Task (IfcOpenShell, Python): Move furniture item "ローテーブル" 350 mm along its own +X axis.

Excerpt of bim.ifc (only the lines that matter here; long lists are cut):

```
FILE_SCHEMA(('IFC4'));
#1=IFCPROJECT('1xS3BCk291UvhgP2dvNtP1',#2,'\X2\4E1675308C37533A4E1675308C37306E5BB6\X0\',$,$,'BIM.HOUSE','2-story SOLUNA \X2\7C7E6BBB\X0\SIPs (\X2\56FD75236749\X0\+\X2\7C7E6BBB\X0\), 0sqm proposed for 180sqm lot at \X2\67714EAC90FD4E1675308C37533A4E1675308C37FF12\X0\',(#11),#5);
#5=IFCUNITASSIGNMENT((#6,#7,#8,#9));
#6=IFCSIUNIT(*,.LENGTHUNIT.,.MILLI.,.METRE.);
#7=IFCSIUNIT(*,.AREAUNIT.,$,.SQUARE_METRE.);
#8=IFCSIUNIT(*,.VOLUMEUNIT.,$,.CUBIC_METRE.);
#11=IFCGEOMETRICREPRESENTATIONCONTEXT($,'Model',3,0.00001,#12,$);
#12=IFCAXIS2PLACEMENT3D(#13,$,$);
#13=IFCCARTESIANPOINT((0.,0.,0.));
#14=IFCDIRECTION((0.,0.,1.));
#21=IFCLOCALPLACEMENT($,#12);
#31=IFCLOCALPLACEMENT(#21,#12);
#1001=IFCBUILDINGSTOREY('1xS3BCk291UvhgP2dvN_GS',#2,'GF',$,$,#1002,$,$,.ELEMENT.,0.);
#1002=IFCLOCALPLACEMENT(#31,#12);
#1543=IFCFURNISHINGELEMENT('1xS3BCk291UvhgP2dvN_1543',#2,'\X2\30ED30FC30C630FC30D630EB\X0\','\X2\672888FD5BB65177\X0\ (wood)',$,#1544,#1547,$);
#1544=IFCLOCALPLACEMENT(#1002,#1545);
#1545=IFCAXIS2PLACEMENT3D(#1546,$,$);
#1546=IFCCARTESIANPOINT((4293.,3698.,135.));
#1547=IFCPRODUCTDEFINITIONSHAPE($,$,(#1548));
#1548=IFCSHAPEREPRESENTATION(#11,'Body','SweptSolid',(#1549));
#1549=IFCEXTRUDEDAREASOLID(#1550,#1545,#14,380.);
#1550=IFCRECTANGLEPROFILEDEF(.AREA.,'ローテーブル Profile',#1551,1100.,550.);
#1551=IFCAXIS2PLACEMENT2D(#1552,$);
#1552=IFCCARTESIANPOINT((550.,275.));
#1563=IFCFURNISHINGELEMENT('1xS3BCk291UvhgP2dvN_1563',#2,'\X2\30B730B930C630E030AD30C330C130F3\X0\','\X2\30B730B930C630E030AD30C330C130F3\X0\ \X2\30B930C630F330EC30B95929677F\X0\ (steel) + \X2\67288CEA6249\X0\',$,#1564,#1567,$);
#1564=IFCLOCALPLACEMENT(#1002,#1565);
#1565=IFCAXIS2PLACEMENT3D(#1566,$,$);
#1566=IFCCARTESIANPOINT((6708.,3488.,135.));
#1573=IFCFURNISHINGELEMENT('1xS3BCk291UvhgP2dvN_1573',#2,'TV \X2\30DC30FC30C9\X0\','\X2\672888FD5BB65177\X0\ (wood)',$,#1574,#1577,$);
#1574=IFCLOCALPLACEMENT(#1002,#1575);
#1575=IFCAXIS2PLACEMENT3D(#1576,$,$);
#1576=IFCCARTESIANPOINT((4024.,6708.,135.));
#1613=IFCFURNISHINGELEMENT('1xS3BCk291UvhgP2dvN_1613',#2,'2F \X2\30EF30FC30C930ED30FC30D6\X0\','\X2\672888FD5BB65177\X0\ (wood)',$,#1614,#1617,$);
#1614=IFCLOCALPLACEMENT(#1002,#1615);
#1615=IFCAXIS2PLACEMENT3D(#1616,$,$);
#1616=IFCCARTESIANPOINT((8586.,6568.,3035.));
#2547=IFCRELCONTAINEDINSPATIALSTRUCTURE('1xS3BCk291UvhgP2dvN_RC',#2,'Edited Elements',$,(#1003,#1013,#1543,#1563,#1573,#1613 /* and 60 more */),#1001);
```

```python
import ifcopenshell
import ifcopenshell.api.geometry
import ifcopenshell.util.placement

model = ifcopenshell.open("bim.ifc")

item = model.by_guid("1xS3BCk291UvhgP2dvN_1543")
matrix = ifcopenshell.util.placement.get_local_placement(item.ObjectPlacement)
matrix[:3, 3] += matrix[:3, 0] * 350.0
ifcopenshell.api.geometry.edit_object_placement(model, product=item, matrix=matrix, is_si=False)

print(ifcopenshell.util.placement.get_local_placement(item.ObjectPlacement).round(3) + 0.0)

model.write("bim-out.ifc")
```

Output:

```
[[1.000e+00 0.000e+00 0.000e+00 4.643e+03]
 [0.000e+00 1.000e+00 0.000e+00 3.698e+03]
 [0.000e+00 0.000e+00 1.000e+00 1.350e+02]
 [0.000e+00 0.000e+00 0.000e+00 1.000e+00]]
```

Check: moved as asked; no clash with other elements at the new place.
